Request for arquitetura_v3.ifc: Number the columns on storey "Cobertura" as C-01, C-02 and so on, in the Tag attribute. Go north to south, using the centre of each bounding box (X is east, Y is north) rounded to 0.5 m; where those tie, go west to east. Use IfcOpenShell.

First a look at what the model holds.

```python
import ifcopenshell
import ifcopenshell.util.element
import ifcopenshell.util.placement

model = ifcopenshell.open("arquitetura_v3.ifc")
print(model.schema)
storey = next(s for s in model.by_type("IfcBuildingStorey") if s.Name == "Cobertura")
columns = [e for e in ifcopenshell.util.element.get_decomposition(storey) if e.is_a("IfcColumn")]
for e in sorted(columns, key=lambda e: e.id()):
    origin = ifcopenshell.util.placement.get_local_placement(e.ObjectPlacement)[:3, 3]
    print(e.id(), e.Tag, e.Name, origin.round(2) + 0.0, sep=" | ")
```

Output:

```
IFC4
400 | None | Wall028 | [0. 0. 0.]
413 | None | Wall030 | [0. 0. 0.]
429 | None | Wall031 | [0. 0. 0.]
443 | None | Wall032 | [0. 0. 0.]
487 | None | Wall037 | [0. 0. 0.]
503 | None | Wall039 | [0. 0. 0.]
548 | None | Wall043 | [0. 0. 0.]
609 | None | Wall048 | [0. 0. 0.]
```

```python
import ifcopenshell
import ifcopenshell.geom
import ifcopenshell.util.element
import ifcopenshell.util.shape

model = ifcopenshell.open("arquitetura_v3.ifc")
settings = ifcopenshell.geom.settings()
settings.set("use-world-coords", True)


def centre(element):
    shape = ifcopenshell.geom.create_shape(settings, element)
    return ifcopenshell.util.shape.get_bbox_centroid(shape.geometry)


storey = next(s for s in model.by_type("IfcBuildingStorey") if s.Name == "Cobertura")
columns = [e for e in ifcopenshell.util.element.get_decomposition(storey) if e.is_a("IfcColumn")]

# Insertion points can sit at a corner or the storey origin, so sort by the geometry (in metres).
centres = {e: centre(e) for e in columns}
columns.sort(key=lambda e: (-round(centres[e][1] / 0.5), centres[e][0]))

for i, e in enumerate(columns, start=1):
    number = f"C-{i:02d}"
    e.Tag = number
    print(e.id(), number)

model.write("arquitetura_v3_updated.ifc")
```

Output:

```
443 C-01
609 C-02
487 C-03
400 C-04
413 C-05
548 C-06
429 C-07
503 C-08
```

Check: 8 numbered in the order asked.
